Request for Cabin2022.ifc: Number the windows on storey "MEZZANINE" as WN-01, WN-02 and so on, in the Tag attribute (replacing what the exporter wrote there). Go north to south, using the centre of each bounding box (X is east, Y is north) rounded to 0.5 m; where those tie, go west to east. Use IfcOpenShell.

First a look at what the model holds.

```python
import ifcopenshell
import ifcopenshell.util.element
import ifcopenshell.util.placement

model = ifcopenshell.open("Cabin2022.ifc")
print(model.schema)
storey = next(s for s in model.by_type("IfcBuildingStorey") if s.Name == "MEZZANINE")
windows = [e for e in ifcopenshell.util.element.get_decomposition(storey) if e.is_a("IfcWindow")]
for e in sorted(windows, key=lambda e: e.id()):
    origin = ifcopenshell.util.placement.get_local_placement(e.ObjectPlacement)[:3, 3]
    print(e.id(), e.Tag, e.Name, origin.round(2) + 0.0, sep=" | ")
```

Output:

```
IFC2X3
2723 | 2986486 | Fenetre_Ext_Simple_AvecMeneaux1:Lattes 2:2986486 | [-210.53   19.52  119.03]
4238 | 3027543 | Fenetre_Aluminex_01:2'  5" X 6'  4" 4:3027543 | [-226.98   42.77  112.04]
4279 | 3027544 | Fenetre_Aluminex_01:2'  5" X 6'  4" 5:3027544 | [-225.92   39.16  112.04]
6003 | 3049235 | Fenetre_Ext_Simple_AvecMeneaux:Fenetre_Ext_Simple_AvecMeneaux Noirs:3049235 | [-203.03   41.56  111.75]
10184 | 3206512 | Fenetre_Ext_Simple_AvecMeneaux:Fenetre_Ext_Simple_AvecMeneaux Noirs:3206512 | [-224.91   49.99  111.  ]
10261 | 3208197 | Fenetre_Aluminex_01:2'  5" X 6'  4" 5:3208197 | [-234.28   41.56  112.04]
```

```python
import ifcopenshell
import ifcopenshell.geom
import ifcopenshell.util.element
import ifcopenshell.util.shape

model = ifcopenshell.open("Cabin2022.ifc")
settings = ifcopenshell.geom.settings()
settings.set("use-world-coords", True)


def centre(element):
    shape = ifcopenshell.geom.create_shape(settings, element)
    return ifcopenshell.util.shape.get_bbox_centroid(shape.geometry)


storey = next(s for s in model.by_type("IfcBuildingStorey") if s.Name == "MEZZANINE")
windows = [e for e in ifcopenshell.util.element.get_decomposition(storey) if e.is_a("IfcWindow")]

# Insertion points can sit at a corner or the storey origin, so sort by the geometry (in metres).
centres = {e: centre(e) for e in windows}
windows.sort(key=lambda e: (-round(centres[e][1] / 0.5), centres[e][0]))

for i, e in enumerate(windows, start=1):
    number = f"WN-{i:02d}"
    e.Tag = number
    print(e.id(), number)

model.write("Cabin2022_edited.ifc")
```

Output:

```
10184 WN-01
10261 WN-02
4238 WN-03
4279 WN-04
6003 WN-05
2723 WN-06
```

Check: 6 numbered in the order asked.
